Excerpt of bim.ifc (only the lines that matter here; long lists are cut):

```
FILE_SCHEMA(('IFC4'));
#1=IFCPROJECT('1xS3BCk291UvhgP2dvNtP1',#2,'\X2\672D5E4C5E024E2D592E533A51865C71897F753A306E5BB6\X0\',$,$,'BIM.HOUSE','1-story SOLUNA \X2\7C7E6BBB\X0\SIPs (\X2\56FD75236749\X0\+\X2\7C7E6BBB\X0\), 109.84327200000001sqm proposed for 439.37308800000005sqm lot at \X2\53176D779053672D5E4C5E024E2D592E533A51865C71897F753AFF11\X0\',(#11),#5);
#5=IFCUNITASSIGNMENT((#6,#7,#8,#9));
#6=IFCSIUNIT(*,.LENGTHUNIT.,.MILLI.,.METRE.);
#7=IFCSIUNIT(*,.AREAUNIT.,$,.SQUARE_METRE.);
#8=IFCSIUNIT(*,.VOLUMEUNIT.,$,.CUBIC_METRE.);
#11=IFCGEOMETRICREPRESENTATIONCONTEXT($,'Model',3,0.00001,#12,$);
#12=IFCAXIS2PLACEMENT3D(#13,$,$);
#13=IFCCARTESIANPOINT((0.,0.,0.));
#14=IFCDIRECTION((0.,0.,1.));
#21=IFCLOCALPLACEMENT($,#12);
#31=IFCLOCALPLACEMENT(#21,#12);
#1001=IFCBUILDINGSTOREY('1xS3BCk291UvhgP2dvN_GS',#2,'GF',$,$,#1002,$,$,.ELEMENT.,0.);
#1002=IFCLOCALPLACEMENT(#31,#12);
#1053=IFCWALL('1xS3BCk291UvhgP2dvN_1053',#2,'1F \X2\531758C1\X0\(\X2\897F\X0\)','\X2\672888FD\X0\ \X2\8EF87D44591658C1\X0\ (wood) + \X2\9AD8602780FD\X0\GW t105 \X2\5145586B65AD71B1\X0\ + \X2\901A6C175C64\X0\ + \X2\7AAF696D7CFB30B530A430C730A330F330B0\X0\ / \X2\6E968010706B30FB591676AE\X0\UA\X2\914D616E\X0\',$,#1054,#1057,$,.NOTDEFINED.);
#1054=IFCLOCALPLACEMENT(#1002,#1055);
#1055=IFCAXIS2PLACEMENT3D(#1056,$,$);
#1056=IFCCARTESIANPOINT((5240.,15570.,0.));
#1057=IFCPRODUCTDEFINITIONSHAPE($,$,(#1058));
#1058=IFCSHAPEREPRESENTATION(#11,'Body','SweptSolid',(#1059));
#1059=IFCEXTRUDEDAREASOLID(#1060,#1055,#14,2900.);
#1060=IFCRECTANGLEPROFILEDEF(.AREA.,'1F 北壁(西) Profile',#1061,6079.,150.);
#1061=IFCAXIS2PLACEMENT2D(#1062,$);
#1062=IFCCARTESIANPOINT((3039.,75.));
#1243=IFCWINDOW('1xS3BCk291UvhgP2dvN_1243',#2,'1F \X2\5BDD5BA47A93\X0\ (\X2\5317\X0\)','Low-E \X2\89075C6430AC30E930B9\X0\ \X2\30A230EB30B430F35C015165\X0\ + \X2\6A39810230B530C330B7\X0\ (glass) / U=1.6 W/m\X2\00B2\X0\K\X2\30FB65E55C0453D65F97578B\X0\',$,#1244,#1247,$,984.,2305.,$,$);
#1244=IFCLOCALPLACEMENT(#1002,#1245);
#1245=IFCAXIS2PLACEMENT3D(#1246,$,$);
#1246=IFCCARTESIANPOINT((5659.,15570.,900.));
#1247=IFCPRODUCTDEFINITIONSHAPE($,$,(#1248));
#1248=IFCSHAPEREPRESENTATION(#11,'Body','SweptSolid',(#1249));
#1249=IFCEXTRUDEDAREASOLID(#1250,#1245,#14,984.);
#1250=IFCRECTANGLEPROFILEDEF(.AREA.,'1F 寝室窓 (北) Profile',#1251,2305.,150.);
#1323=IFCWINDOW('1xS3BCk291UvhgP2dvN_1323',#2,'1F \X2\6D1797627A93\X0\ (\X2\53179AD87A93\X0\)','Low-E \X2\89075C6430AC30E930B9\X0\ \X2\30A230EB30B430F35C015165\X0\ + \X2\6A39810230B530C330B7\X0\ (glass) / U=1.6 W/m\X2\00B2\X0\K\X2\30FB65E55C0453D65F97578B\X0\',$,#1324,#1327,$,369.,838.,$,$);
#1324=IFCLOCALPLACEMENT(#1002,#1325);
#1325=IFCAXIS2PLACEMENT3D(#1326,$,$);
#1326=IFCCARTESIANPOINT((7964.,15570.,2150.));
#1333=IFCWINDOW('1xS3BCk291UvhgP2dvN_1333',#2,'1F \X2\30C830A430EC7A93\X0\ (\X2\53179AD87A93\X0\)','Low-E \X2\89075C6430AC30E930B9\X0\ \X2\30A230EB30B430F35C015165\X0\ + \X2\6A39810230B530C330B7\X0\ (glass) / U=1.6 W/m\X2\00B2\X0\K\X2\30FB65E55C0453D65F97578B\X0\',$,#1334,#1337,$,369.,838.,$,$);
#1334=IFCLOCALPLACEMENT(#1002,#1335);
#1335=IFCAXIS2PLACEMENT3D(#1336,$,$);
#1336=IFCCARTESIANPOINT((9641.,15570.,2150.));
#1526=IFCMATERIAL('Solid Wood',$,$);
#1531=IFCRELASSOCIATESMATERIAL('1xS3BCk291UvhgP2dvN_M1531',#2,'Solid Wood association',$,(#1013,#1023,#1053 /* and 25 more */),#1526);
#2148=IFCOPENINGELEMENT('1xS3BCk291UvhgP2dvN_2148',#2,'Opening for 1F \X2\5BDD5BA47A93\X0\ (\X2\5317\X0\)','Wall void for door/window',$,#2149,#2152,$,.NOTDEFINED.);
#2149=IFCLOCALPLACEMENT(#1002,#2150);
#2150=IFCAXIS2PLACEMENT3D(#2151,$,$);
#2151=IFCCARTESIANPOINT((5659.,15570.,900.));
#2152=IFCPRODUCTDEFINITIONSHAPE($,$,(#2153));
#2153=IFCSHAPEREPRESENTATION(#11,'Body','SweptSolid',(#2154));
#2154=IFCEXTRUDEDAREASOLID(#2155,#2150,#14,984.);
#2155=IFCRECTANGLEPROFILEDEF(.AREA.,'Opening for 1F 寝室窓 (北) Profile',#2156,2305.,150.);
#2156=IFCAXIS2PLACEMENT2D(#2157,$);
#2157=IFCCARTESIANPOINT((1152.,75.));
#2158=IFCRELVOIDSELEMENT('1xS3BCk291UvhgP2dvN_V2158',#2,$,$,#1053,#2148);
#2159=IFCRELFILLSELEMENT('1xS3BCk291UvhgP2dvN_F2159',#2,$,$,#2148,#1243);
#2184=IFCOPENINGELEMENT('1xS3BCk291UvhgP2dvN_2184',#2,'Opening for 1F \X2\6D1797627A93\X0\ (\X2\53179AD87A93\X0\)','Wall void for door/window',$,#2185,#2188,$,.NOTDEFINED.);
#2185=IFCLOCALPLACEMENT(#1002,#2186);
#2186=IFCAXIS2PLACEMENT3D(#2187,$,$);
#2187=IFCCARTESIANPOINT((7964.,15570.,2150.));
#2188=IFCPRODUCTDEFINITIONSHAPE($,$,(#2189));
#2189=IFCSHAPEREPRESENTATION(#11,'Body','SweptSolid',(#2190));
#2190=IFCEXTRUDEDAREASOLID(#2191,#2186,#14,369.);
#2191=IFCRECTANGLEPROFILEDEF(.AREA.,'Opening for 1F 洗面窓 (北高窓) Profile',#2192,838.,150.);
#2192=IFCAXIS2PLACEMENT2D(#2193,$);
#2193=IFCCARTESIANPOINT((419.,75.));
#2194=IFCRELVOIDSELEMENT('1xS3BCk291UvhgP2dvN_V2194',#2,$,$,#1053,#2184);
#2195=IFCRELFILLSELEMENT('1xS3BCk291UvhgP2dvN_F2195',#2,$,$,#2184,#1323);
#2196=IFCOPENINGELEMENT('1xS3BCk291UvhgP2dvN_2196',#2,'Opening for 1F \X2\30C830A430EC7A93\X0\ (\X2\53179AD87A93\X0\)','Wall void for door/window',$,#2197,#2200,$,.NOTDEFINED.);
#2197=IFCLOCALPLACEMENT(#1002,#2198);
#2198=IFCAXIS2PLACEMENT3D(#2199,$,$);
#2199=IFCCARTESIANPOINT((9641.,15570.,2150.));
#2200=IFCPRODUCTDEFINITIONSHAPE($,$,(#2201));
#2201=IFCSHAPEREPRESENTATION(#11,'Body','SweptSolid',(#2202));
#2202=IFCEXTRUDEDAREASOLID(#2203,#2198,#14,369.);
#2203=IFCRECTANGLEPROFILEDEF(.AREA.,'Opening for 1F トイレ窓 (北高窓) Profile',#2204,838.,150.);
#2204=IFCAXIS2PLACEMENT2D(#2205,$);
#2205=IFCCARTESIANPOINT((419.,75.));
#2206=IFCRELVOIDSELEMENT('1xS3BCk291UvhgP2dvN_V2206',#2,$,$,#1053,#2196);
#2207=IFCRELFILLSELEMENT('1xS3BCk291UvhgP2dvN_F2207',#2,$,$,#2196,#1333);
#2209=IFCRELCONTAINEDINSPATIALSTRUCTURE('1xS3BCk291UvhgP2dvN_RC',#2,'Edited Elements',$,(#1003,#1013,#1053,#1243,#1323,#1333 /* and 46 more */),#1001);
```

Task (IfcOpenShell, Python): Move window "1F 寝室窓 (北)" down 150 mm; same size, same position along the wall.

```python
import numpy as np
import ifcopenshell
import ifcopenshell.api.geometry
import ifcopenshell.util.placement
import ifcopenshell.util.unit

model = ifcopenshell.open("bim.ifc")
unit_scale = ifcopenshell.util.unit.calculate_unit_scale(model)

window = model.by_guid("1xS3BCk291UvhgP2dvN_1243")
opening = window.FillsVoids[0].RelatingOpeningElement
dz = -0.15 / unit_scale

shift = np.array([0.0, 0.0, dz])
# The window is not placed relative to its opening, so move both.
for product in (opening, window):
    matrix = ifcopenshell.util.placement.get_local_placement(product.ObjectPlacement)
    matrix[:3, 3] += shift
    ifcopenshell.api.geometry.edit_object_placement(model, product=product, matrix=matrix, is_si=False)

print(f"moved by {dz * unit_scale:+.3f} m")

model.write("bim_rev.ifc")
```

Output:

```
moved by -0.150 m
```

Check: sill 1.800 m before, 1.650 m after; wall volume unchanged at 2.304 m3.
